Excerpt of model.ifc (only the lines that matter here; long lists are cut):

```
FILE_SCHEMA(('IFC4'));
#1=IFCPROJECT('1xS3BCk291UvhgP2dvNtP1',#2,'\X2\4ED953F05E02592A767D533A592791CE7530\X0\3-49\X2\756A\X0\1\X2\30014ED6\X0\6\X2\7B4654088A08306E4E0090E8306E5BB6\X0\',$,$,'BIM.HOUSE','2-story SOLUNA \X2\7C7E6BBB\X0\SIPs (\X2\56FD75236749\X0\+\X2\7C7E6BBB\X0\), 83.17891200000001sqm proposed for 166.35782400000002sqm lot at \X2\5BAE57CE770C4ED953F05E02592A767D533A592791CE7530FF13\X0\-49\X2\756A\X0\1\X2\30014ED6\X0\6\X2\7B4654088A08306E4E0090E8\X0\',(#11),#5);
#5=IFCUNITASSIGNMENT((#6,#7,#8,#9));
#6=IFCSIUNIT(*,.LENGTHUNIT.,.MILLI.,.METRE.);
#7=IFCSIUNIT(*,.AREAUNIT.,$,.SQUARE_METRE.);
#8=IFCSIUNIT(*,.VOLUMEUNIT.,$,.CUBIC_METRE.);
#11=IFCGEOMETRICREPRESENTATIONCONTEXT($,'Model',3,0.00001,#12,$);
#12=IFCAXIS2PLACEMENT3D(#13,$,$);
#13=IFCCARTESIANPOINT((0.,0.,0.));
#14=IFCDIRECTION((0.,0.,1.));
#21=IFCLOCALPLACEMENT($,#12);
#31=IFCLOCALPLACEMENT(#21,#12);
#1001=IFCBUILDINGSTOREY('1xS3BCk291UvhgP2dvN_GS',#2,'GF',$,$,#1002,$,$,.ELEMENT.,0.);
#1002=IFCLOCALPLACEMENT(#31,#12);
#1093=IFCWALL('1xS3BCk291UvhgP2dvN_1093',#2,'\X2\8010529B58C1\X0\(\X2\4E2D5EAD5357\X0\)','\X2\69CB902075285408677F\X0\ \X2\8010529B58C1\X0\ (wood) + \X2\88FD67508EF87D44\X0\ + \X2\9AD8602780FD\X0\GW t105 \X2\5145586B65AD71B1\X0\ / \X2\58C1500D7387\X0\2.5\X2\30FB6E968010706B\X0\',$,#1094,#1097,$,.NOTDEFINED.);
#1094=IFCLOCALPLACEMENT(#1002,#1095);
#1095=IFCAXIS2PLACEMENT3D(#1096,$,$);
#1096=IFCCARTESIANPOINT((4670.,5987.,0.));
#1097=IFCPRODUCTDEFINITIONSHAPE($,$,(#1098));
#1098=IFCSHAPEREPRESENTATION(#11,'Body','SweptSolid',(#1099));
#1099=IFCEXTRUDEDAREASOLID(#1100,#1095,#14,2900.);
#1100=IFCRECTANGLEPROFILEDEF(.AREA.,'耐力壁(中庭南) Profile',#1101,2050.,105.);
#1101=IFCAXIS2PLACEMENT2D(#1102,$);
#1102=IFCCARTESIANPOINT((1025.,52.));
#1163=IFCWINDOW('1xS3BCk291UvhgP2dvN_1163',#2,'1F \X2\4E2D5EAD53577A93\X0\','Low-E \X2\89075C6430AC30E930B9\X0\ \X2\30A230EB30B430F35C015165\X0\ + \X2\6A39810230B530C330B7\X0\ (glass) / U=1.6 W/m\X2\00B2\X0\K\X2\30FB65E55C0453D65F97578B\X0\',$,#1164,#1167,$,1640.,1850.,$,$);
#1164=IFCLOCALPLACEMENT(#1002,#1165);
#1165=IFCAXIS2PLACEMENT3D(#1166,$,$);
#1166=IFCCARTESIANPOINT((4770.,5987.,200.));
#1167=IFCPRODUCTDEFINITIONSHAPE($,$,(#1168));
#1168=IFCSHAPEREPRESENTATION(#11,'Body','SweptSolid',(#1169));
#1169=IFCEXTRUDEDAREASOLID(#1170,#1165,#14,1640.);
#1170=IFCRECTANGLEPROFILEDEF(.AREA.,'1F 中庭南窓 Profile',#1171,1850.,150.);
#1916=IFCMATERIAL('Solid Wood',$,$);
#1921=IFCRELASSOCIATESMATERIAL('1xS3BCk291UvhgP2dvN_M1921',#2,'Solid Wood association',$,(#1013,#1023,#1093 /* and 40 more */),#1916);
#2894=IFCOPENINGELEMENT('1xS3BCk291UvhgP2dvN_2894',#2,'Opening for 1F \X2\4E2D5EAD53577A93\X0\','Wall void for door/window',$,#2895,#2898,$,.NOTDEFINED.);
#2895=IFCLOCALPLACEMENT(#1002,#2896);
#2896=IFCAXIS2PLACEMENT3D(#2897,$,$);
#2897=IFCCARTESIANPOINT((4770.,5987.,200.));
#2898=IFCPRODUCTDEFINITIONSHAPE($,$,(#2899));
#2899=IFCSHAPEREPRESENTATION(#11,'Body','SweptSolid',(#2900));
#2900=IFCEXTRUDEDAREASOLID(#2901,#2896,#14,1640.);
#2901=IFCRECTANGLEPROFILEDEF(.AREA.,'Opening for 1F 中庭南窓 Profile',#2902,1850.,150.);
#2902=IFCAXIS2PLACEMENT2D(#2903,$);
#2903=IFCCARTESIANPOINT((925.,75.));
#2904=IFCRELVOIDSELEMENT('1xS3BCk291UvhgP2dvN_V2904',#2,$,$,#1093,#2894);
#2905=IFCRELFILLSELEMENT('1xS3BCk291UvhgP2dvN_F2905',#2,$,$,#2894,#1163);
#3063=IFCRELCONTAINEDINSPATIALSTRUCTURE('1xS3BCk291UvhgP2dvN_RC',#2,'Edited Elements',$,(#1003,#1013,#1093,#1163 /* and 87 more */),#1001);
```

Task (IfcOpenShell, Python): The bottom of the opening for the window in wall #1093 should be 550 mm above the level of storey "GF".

```python
import numpy as np
import ifcopenshell
import ifcopenshell.api.geometry
import ifcopenshell.geom
import ifcopenshell.util.element
import ifcopenshell.util.placement
import ifcopenshell.util.shape
import ifcopenshell.util.unit

model = ifcopenshell.open("model.ifc")
unit_scale = ifcopenshell.util.unit.calculate_unit_scale(model)

window = model.by_id(1163)
opening = window.FillsVoids[0].RelatingOpeningElement
storey = ifcopenshell.util.element.get_container(window, ifc_class="IfcBuildingStorey")
level = ifcopenshell.util.placement.get_local_placement(storey.ObjectPlacement)[2, 3]

# The opening's origin need not be at the sill, so measure its lowest point.
shape = ifcopenshell.geom.create_shape(ifcopenshell.geom.settings(), opening)
bottom = ifcopenshell.util.shape.get_shape_bottom_elevation(shape, shape.geometry) / unit_scale
dz = level + 550.0 - bottom

shift = np.array([0.0, 0.0, dz])
# The window is not placed relative to its opening, so move both.
for product in (opening, window):
    matrix = ifcopenshell.util.placement.get_local_placement(product.ObjectPlacement)
    matrix[:3, 3] += shift
    ifcopenshell.api.geometry.edit_object_placement(model, product=product, matrix=matrix, is_si=False)

print(f"moved by {dz * unit_scale:+.3f} m")

model.write("model_updated.ifc")
```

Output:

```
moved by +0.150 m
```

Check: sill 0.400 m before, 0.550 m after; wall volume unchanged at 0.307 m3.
